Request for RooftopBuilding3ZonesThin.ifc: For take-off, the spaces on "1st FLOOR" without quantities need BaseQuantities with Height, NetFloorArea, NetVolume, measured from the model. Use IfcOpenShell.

First a look at what the model holds.

```python
import ifcopenshell
import ifcopenshell.util.element
import ifcopenshell.util.unit

model = ifcopenshell.open("RooftopBuilding3ZonesThin.ifc")
print(model.schema)
for unit_type in ("LENGTHUNIT", "AREAUNIT", "VOLUMEUNIT"):
    print(unit_type, ifcopenshell.util.unit.calculate_unit_scale(model, unit_type))
storey = next(s for s in model.by_type("IfcBuildingStorey") if s.Name == "1st FLOOR")
spaces = [e for e in ifcopenshell.util.element.get_decomposition(storey) if e.is_a("IfcSpace")]
for e in sorted(spaces, key=lambda e: e.id()):
    print(e.id(), e.is_a(), e.Name, list(ifcopenshell.util.element.get_psets(e, qtos_only=True)), sep=" | ")
```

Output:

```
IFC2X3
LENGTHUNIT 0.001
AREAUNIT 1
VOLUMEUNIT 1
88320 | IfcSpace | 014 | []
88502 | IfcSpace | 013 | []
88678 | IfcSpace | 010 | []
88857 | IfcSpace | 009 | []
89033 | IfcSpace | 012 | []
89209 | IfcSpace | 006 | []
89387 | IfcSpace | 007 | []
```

```python
import ifcopenshell
import ifcopenshell.api.pset
import ifcopenshell.geom
import ifcopenshell.util.element
import ifcopenshell.util.shape
import ifcopenshell.util.unit

model = ifcopenshell.open("RooftopBuilding3ZonesThin.ifc")
unit_scale = ifcopenshell.util.unit.calculate_unit_scale(model)
area_scale = ifcopenshell.util.unit.calculate_unit_scale(model, "AREAUNIT")
volume_scale = ifcopenshell.util.unit.calculate_unit_scale(model, "VOLUMEUNIT")
settings = ifcopenshell.geom.settings()

storey = next(s for s in model.by_type("IfcBuildingStorey") if s.Name == "1st FLOOR")
spaces = [e for e in ifcopenshell.util.element.get_decomposition(storey) if e.is_a("IfcSpace")]

for e in sorted(spaces, key=lambda e: e.id()):
    if ifcopenshell.util.element.get_psets(e, qtos_only=True, should_inherit=False):
        continue
    # Geometry comes back in metres, in the element's own axes.
    shape = ifcopenshell.geom.create_shape(settings, e)
    values = {
        "Height": ifcopenshell.util.shape.get_z(shape.geometry) / unit_scale,
        "NetFloorArea": ifcopenshell.util.shape.get_footprint_area(shape.geometry) / area_scale,
        "NetVolume": ifcopenshell.util.shape.get_volume(shape.geometry) / volume_scale,
    }
    qto = ifcopenshell.api.pset.add_qto(model, product=e, name="BaseQuantities")
    ifcopenshell.api.pset.edit_qto(model, qto=qto, properties=values)
    print(e.id(), {k: round(v, 3) for k, v in values.items()})

model.write("RooftopBuilding3ZonesThin_edited.ifc")
```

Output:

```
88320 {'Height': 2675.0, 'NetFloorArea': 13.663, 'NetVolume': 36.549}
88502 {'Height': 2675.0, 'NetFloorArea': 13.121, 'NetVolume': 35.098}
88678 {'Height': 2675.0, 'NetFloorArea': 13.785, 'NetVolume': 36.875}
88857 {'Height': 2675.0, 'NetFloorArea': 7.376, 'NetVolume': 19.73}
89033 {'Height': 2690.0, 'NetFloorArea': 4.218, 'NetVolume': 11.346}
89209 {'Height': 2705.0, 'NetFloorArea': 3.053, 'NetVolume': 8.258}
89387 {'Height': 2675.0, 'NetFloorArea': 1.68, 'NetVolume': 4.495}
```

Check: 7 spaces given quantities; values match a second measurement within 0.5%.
